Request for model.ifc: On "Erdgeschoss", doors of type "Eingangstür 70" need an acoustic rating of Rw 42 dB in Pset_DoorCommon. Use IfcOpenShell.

First a look at what the model holds.

```python
import ifcopenshell
import ifcopenshell.util.element

model = ifcopenshell.open("model.ifc")
print(model.schema)
storey = next(s for s in model.by_type("IfcBuildingStorey") if s.Name == "Erdgeschoss")
doors = [e for e in ifcopenshell.util.element.get_decomposition(storey) if e.is_a("IfcDoor")]
seen = {}
for e in doors:
    element_type = ifcopenshell.util.element.get_type(e)
    key = (element_type.Name if element_type != e and element_type else None, ifcopenshell.util.element.get_pset(e, "Pset_DoorCommon", "AcousticRating"))
    seen[key] = seen.get(key, 0) + 1
for (name, value), count in sorted(seen.items(), key=str):
    print(count, "x", name, "|", value)
```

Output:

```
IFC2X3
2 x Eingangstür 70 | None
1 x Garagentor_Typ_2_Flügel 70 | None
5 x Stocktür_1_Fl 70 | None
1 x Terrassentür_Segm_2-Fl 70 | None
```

```python
import ifcopenshell
import ifcopenshell.api.pset
import ifcopenshell.util.element

model = ifcopenshell.open("model.ifc")

storey = next(s for s in model.by_type("IfcBuildingStorey") if s.Name == "Erdgeschoss")
doors = [e for e in ifcopenshell.util.element.get_decomposition(storey) if e.is_a("IfcDoor")]

count = 0
for e in doors:
    element_type = ifcopenshell.util.element.get_type(e)
    if element_type in (None, e) or element_type.Name != "Eingangstür 70":
        continue
    # add_pset returns the element's existing set when there is one.
    pset = ifcopenshell.api.pset.add_pset(model, product=e, name="Pset_DoorCommon")
    ifcopenshell.api.pset.edit_pset(model, pset=pset, properties={"AcousticRating": "Rw 42 dB"})
    count += 1

print(count, "doors updated")

model.write("model-out.ifc")
```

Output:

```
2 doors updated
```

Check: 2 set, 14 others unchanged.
